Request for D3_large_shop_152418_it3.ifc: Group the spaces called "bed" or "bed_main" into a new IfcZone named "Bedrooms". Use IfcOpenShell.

First a look at what the model holds.

```python
import ifcopenshell

model = ifcopenshell.open("D3_large_shop_152418_it3.ifc")
print(model.schema)
seen = {}
for space in model.by_type("IfcSpace"):
    seen[space.LongName] = seen.get(space.LongName, 0) + 1
for name, count in sorted(seen.items(), key=str):
    print(count, "x", name)
print("zones:", [z.Name for z in model.by_type("IfcZone")][:20])
```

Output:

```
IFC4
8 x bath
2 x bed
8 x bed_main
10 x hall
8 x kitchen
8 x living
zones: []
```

```python
import ifcopenshell
import ifcopenshell.api.group
import ifcopenshell.api.root

model = ifcopenshell.open("D3_large_shop_152418_it3.ifc")

names = {"bed", "bed_main"}
spaces = [s for s in model.by_type("IfcSpace") if s.LongName in names]

zone = ifcopenshell.api.root.create_entity(model, ifc_class="IfcZone", name="Bedrooms")
ifcopenshell.api.group.assign_group(model, products=spaces, group=zone)
print(len(spaces), "spaces in", zone.Name)

model.write("D3_large_shop_152418_it3_updated.ifc")
```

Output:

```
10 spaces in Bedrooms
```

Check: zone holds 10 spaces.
